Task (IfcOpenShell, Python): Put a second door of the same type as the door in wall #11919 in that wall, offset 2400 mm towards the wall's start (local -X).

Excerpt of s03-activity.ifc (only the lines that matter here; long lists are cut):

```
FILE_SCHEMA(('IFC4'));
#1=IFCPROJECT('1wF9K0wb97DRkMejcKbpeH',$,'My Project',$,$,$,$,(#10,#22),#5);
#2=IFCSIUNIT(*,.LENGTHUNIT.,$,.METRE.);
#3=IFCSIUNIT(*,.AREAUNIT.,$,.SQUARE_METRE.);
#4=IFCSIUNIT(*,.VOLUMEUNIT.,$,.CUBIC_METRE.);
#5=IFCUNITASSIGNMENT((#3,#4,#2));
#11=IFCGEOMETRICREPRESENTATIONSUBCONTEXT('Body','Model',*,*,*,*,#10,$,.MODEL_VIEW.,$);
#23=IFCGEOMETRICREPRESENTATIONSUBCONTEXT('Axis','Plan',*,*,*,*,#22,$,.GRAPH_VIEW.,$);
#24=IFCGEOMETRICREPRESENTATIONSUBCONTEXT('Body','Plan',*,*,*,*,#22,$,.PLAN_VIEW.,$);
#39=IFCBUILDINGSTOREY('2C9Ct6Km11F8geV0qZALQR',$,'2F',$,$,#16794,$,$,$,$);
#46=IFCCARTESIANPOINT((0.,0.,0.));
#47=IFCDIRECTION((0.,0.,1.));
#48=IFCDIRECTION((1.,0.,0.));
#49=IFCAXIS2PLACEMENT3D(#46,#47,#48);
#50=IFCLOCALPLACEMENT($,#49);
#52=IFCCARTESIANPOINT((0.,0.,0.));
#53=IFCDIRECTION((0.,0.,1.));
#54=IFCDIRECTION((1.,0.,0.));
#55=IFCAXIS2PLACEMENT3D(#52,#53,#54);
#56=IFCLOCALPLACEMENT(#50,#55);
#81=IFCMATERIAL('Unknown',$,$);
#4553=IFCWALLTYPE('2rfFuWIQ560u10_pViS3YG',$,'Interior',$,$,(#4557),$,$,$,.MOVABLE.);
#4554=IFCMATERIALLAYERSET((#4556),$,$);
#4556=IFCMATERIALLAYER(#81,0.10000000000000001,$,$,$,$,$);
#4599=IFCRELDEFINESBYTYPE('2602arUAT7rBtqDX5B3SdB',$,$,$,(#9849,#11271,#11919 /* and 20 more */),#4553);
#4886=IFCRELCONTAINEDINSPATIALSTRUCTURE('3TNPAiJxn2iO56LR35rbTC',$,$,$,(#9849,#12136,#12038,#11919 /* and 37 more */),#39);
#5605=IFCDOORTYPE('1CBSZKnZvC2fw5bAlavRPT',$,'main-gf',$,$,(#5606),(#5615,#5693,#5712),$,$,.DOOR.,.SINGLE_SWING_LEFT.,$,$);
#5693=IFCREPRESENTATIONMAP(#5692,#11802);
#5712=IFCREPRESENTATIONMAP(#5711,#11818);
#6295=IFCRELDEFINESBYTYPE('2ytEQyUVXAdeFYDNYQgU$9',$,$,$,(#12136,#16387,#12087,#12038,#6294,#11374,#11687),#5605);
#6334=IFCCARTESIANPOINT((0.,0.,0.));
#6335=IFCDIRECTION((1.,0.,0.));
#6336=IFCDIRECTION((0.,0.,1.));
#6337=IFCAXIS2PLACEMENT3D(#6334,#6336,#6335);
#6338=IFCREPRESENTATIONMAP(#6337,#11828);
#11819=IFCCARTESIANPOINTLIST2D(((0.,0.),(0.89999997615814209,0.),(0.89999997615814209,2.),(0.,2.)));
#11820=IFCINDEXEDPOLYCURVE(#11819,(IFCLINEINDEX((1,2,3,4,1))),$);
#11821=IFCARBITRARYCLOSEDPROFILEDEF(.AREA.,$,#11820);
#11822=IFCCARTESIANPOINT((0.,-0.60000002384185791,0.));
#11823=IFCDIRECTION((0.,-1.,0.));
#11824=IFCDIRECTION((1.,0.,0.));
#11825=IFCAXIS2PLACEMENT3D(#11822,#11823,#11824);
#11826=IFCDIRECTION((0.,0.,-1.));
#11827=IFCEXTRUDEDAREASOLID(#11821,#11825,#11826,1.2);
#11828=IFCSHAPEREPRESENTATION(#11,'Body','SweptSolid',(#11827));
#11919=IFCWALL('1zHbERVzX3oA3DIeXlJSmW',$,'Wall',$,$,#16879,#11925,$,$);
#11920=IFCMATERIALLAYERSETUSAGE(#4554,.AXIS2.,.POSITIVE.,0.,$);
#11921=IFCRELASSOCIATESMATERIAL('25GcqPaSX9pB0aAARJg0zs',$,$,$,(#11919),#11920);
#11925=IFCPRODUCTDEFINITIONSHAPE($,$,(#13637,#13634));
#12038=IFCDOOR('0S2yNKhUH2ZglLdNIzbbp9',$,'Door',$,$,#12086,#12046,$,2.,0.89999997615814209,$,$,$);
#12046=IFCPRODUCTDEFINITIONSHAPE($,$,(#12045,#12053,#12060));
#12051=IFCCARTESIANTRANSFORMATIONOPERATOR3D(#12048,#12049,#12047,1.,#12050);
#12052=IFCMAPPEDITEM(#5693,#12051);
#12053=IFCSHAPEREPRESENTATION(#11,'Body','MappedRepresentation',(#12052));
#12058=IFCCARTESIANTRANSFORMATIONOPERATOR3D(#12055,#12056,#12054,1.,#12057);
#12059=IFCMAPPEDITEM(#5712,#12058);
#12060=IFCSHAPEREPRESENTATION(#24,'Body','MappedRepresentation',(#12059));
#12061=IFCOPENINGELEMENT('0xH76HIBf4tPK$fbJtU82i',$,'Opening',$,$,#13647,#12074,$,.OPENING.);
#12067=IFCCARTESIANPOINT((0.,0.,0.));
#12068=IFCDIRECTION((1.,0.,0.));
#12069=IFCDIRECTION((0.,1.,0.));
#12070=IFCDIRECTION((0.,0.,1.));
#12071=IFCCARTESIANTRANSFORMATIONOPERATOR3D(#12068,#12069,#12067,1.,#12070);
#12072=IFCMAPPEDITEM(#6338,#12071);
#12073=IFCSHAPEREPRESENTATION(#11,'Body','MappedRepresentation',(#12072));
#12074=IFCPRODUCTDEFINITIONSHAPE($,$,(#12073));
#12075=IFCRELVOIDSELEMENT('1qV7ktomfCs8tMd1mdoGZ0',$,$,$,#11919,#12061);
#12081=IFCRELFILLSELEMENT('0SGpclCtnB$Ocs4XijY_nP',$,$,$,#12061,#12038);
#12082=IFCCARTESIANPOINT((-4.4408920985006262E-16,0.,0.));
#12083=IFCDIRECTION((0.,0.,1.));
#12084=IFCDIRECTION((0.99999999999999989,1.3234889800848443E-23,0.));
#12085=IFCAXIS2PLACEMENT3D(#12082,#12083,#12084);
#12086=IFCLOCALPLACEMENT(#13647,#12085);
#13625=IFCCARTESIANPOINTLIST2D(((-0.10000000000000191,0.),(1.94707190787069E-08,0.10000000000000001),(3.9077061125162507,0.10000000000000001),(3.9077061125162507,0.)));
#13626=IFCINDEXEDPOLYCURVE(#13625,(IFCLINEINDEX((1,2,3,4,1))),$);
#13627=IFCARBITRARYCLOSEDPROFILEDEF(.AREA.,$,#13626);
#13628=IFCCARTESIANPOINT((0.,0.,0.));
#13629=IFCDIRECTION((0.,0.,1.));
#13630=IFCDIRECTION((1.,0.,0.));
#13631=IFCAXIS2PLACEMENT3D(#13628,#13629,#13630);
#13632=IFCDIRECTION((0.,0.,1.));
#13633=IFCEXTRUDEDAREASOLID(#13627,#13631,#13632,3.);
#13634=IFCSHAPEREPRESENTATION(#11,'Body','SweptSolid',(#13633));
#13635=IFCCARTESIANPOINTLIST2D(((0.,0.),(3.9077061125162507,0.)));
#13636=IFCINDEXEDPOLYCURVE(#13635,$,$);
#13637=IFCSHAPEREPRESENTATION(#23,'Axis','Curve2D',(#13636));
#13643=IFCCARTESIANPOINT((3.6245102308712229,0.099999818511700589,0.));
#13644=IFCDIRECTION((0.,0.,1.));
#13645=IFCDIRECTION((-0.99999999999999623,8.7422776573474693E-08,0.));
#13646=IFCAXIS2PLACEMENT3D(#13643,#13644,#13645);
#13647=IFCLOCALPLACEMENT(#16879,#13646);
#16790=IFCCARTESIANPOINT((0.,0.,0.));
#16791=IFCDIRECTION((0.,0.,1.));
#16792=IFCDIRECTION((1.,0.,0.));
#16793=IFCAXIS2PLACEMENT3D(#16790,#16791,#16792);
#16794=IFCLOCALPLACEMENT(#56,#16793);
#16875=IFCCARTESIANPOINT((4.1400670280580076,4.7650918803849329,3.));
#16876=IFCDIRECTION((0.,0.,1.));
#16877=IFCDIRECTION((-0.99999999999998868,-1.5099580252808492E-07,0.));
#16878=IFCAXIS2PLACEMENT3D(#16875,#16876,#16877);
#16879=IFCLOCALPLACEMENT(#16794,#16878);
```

```python
import ifcopenshell
import ifcopenshell.api.feature
import ifcopenshell.api.geometry
import ifcopenshell.api.root
import ifcopenshell.geom
import ifcopenshell.util.element
import ifcopenshell.util.placement
import ifcopenshell.util.shape
import ifcopenshell.util.unit

model = ifcopenshell.open("s03-activity.ifc")
unit_scale = ifcopenshell.util.unit.calculate_unit_scale(model)
settings = ifcopenshell.geom.settings()


def volume(element):
    """Net volume in cubic metres, openings subtracted."""
    shape = ifcopenshell.geom.create_shape(settings, element)
    return ifcopenshell.util.shape.get_volume(shape.geometry)


door = model.by_id(12038)
opening = door.FillsVoids[0].RelatingOpeningElement
wall = opening.VoidsElements[0].RelatingBuildingElement
before = volume(wall)
shift = ifcopenshell.util.placement.get_local_placement(wall.ObjectPlacement)[:3, 0] * -2.4 / unit_scale

# copy_class copies the void relationship, type, container and properties, but no geometry.
new_opening = ifcopenshell.api.root.copy_class(model, product=opening)
new_opening.Representation = ifcopenshell.util.element.copy_deep(
    model, opening.Representation, exclude=["IfcGeometricRepresentationContext", "IfcRepresentationMap"]
)
new_door = ifcopenshell.api.root.copy_class(model, product=door)
new_door.Representation = ifcopenshell.util.element.copy_deep(
    model, door.Representation, exclude=["IfcGeometricRepresentationContext", "IfcRepresentationMap"]
)
ifcopenshell.api.feature.add_filling(model, opening=new_opening, element=new_door)

for old, new in ((opening, new_opening), (door, new_door)):
    matrix = ifcopenshell.util.placement.get_local_placement(old.ObjectPlacement)
    matrix[:3, 3] += shift
    ifcopenshell.api.geometry.edit_object_placement(model, product=new, matrix=matrix, is_si=False)

after = volume(wall)

print(f"wall volume {before:.3f} -> {after:.3f} m3")

model.write("s03-activity_v2.ifc")
```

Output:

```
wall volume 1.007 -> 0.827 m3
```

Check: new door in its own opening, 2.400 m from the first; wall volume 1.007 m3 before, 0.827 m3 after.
